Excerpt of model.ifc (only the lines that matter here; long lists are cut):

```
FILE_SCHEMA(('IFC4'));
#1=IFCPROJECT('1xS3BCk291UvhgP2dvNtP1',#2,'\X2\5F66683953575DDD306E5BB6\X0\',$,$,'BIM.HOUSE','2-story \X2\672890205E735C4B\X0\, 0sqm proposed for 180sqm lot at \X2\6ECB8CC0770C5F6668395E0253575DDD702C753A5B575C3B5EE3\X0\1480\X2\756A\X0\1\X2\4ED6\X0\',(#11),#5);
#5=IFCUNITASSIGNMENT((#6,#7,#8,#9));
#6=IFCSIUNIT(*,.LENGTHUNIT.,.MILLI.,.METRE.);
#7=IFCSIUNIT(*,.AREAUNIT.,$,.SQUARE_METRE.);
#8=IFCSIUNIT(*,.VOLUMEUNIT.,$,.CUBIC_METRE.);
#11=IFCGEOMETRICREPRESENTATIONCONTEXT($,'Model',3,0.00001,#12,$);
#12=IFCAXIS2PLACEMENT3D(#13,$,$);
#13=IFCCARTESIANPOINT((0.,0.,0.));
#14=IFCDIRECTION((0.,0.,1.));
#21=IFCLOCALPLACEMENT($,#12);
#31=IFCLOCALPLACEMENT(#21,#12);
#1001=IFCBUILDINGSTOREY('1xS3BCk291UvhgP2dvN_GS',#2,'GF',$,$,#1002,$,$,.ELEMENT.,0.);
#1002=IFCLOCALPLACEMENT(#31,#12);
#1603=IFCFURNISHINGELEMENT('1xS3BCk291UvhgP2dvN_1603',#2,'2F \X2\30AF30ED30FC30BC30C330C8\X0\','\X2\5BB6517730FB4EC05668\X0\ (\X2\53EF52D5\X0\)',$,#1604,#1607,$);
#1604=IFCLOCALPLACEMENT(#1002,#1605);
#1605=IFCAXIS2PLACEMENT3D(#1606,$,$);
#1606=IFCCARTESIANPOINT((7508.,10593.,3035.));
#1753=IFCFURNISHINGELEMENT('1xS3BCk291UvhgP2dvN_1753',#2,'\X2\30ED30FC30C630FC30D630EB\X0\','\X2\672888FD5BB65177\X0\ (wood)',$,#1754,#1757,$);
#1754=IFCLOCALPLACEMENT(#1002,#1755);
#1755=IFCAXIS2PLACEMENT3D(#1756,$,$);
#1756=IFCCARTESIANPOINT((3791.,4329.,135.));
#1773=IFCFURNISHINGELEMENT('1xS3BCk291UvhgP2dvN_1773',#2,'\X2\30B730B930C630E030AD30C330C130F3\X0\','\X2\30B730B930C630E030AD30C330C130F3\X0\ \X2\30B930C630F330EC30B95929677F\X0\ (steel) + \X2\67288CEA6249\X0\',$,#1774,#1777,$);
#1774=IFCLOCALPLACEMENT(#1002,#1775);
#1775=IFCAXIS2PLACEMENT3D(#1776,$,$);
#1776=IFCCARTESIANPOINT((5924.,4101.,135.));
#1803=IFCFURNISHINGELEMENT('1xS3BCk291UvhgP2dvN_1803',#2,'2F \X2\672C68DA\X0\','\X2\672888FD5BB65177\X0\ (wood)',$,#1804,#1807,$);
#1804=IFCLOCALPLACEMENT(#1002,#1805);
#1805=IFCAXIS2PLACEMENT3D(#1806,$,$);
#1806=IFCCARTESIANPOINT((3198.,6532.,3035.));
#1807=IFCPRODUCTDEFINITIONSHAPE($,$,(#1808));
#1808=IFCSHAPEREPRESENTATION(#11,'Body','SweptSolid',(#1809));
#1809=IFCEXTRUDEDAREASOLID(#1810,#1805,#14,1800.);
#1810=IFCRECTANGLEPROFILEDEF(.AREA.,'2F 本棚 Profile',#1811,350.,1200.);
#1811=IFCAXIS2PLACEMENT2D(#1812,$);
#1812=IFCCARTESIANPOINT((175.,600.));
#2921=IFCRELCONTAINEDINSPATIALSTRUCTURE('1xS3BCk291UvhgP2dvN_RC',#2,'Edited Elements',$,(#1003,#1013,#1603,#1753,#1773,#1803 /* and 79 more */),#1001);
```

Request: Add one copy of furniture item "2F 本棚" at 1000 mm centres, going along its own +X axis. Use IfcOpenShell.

```python
import ifcopenshell
import ifcopenshell.api.geometry
import ifcopenshell.api.root
import ifcopenshell.util.element
import ifcopenshell.util.placement
import ifcopenshell.util.unit

model = ifcopenshell.open("model.ifc")
unit_scale = ifcopenshell.util.unit.calculate_unit_scale(model)


def reuse_history(source, copy):
    """copy_class also copies each property set's owner history, people and application; keep the originals."""
    for rel in copy.IsDefinedBy:
        if rel.is_a("IfcRelDefinesByProperties") and (history := rel.RelatingPropertyDefinition.OwnerHistory):
            rel.RelatingPropertyDefinition.OwnerHistory = source.OwnerHistory
            ifcopenshell.util.element.remove_deep2(model, history)


source = model.by_guid("1xS3BCk291UvhgP2dvN_1803")
base = ifcopenshell.util.placement.get_local_placement(source.ObjectPlacement)
step = base[:3, 0] * 1 / unit_scale

for i in range(1, 2):
    copy = ifcopenshell.api.root.copy_class(model, product=source)
    copy.Representation = ifcopenshell.util.element.copy_deep(
        model, source.Representation, exclude=["IfcGeometricRepresentationContext", "IfcRepresentationMap"]
    )
    reuse_history(source, copy)
    matrix = base.copy()
    matrix[:3, 3] += i * step
    print("added at", matrix[:3, 3].round(3) + 0.0)
    ifcopenshell.api.geometry.edit_object_placement(model, product=copy, matrix=matrix, is_si=False)

model.write("model_edited.ifc")
```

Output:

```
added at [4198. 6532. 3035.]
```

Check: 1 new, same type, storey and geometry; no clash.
